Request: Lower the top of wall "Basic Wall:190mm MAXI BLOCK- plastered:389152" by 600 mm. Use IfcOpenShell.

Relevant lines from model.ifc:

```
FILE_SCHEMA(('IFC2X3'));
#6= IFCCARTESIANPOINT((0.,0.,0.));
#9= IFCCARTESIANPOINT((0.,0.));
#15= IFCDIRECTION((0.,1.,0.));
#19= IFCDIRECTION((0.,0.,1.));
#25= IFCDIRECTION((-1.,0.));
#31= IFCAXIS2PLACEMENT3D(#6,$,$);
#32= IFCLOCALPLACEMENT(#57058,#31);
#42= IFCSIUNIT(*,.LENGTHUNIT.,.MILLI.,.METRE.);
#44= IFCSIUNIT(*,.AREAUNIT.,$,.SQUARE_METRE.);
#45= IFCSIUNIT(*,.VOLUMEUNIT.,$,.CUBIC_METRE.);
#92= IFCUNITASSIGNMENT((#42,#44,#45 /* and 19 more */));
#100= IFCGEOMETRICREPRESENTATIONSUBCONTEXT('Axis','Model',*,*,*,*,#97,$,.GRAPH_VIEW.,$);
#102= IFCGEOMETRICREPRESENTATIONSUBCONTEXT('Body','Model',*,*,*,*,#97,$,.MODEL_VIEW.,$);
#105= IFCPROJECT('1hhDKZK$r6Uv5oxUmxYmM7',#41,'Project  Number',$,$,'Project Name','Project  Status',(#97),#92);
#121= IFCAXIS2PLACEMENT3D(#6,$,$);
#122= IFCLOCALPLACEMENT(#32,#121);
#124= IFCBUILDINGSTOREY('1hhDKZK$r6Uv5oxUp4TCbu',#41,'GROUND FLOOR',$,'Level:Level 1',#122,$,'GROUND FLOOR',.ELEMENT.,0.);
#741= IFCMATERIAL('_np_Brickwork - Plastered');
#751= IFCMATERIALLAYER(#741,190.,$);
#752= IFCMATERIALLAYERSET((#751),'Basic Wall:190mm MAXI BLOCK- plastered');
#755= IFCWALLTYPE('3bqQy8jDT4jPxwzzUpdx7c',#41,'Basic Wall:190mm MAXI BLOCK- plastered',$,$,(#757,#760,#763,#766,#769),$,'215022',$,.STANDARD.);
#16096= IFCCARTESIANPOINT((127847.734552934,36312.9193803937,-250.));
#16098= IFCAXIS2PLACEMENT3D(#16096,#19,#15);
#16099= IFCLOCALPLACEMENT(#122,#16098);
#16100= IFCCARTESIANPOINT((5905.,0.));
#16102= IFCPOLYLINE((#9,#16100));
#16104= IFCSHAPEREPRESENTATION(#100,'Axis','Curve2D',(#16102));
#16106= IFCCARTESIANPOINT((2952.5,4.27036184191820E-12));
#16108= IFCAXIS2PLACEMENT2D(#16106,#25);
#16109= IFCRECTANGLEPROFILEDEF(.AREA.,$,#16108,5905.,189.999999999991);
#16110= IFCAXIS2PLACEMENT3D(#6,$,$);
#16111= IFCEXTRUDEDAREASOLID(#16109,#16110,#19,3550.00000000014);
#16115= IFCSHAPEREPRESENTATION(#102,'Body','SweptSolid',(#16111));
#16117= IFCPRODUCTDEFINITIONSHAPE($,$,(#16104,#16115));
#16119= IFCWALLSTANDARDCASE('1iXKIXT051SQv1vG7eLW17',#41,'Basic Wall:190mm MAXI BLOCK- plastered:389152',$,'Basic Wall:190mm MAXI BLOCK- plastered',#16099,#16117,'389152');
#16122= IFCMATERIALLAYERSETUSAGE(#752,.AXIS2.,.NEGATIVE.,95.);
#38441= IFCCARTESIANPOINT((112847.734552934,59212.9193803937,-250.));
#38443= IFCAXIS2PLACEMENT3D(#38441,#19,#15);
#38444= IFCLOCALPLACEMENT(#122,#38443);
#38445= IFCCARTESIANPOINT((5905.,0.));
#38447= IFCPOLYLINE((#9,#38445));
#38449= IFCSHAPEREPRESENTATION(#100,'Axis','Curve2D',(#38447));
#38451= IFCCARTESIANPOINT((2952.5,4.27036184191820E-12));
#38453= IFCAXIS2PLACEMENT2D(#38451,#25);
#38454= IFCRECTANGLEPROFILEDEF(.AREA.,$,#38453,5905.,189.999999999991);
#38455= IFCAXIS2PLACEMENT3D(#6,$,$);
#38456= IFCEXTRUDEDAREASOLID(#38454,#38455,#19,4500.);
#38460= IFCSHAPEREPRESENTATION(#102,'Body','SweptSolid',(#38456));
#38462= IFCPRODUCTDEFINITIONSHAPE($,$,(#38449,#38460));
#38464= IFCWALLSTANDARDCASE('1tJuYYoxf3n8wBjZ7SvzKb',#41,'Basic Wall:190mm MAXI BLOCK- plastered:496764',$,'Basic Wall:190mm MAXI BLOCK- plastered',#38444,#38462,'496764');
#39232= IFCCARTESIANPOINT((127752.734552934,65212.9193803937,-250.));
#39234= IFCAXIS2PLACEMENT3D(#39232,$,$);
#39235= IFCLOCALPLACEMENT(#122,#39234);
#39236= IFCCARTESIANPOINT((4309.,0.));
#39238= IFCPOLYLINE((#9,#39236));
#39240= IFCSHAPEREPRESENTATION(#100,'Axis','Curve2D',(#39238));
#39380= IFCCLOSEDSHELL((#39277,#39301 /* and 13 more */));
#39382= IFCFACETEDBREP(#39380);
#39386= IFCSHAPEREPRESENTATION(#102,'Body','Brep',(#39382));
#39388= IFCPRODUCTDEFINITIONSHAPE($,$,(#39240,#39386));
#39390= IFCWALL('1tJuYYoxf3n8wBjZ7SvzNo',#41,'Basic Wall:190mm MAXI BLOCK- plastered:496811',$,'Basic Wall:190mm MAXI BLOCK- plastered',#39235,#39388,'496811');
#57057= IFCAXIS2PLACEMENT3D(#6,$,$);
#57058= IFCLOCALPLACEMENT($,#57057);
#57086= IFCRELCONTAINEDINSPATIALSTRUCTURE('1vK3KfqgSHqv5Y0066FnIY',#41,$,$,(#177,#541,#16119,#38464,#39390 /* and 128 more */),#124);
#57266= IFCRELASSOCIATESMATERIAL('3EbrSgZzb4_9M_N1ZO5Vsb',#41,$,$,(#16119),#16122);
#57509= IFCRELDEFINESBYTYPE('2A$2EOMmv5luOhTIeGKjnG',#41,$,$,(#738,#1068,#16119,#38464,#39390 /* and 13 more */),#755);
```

```python
import ifcopenshell
import ifcopenshell.geom
import ifcopenshell.util.representation
import ifcopenshell.util.shape

model = ifcopenshell.open("model.ifc")
settings = ifcopenshell.geom.settings()


def volume(element):
    """Net volume in cubic metres, openings subtracted."""
    shape = ifcopenshell.geom.create_shape(settings, element)
    return ifcopenshell.util.shape.get_volume(shape.geometry)


wall = model.by_id(16119)
before = volume(wall)

body = ifcopenshell.util.representation.get_representation(wall, "Model", "Body")
solid = body.Items[0]
old_height = solid.Depth
solid.Depth -= 600.0
after = volume(wall)

print(f"height {old_height:g} -> {solid.Depth:g}, volume {before:.3f} -> {after:.3f} m3")

model.write("model_rev.ifc")
```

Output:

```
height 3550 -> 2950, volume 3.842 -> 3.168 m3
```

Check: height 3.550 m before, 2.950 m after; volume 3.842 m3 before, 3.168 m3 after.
